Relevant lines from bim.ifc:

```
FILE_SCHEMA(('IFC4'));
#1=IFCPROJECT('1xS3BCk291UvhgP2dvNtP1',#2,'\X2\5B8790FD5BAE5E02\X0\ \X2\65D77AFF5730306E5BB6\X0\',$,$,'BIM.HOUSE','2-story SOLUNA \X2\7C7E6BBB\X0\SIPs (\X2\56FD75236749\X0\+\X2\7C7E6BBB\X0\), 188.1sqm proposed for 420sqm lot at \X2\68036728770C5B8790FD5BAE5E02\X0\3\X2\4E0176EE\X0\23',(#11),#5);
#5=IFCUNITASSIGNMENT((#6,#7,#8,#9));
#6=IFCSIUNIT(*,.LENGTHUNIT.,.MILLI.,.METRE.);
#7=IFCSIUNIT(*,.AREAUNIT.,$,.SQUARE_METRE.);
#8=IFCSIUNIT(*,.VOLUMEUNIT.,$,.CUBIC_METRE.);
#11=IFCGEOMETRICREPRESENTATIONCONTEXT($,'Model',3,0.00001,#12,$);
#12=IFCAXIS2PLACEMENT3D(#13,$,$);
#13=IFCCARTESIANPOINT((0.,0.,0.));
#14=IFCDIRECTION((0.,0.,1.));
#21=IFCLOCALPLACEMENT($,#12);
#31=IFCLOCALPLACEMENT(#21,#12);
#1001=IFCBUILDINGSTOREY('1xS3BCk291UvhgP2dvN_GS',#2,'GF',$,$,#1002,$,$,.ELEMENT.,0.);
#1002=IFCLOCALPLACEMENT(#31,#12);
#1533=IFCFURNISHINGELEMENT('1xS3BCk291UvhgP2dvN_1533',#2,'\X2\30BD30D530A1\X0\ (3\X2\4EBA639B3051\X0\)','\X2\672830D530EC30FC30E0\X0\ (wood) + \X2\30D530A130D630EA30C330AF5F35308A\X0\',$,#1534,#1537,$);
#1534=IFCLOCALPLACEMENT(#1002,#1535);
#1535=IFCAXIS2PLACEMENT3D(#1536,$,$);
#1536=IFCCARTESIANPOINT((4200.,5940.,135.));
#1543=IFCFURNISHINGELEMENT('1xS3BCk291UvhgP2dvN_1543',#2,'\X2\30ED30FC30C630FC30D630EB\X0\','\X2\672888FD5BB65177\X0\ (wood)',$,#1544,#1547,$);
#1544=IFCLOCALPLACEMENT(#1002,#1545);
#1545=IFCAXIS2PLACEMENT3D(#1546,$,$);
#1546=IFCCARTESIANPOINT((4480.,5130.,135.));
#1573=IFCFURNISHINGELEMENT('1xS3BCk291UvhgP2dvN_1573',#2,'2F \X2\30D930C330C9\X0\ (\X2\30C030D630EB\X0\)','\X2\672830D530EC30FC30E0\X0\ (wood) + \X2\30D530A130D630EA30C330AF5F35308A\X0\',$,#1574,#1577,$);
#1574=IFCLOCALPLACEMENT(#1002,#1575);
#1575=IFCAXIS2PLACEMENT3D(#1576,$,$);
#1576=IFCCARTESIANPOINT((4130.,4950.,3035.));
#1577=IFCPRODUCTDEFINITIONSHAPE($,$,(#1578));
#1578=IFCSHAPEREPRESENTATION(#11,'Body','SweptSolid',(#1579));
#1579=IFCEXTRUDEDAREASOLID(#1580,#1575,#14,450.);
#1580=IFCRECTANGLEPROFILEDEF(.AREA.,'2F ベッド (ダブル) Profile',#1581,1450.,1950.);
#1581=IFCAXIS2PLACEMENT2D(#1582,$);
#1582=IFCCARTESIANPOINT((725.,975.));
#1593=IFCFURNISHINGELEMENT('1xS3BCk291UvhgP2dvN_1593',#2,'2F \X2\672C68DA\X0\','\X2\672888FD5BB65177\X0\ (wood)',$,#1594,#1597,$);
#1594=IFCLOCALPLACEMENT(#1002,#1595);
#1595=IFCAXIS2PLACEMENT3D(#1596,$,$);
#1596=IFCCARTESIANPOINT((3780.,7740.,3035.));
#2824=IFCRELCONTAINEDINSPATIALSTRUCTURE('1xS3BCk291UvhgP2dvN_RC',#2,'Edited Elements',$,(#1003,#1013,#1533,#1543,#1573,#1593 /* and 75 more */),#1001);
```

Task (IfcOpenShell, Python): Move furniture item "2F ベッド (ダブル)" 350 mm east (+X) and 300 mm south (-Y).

```python
import ifcopenshell
import ifcopenshell.api.geometry
import ifcopenshell.util.placement
import ifcopenshell.util.unit

model = ifcopenshell.open("bim.ifc")
unit_scale = ifcopenshell.util.unit.calculate_unit_scale(model)

item = model.by_guid("1xS3BCk291UvhgP2dvN_1573")
matrix = ifcopenshell.util.placement.get_local_placement(item.ObjectPlacement)
matrix[0, 3] += 0.35 / unit_scale
matrix[1, 3] -= 0.3 / unit_scale
ifcopenshell.api.geometry.edit_object_placement(model, product=item, matrix=matrix, is_si=False)

print(ifcopenshell.util.placement.get_local_placement(item.ObjectPlacement).round(3) + 0.0)

model.write("bim_v2.ifc")
```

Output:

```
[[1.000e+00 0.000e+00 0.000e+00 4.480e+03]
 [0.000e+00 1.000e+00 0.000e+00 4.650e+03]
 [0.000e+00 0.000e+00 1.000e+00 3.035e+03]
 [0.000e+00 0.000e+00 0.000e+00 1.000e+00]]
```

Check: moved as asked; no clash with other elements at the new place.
